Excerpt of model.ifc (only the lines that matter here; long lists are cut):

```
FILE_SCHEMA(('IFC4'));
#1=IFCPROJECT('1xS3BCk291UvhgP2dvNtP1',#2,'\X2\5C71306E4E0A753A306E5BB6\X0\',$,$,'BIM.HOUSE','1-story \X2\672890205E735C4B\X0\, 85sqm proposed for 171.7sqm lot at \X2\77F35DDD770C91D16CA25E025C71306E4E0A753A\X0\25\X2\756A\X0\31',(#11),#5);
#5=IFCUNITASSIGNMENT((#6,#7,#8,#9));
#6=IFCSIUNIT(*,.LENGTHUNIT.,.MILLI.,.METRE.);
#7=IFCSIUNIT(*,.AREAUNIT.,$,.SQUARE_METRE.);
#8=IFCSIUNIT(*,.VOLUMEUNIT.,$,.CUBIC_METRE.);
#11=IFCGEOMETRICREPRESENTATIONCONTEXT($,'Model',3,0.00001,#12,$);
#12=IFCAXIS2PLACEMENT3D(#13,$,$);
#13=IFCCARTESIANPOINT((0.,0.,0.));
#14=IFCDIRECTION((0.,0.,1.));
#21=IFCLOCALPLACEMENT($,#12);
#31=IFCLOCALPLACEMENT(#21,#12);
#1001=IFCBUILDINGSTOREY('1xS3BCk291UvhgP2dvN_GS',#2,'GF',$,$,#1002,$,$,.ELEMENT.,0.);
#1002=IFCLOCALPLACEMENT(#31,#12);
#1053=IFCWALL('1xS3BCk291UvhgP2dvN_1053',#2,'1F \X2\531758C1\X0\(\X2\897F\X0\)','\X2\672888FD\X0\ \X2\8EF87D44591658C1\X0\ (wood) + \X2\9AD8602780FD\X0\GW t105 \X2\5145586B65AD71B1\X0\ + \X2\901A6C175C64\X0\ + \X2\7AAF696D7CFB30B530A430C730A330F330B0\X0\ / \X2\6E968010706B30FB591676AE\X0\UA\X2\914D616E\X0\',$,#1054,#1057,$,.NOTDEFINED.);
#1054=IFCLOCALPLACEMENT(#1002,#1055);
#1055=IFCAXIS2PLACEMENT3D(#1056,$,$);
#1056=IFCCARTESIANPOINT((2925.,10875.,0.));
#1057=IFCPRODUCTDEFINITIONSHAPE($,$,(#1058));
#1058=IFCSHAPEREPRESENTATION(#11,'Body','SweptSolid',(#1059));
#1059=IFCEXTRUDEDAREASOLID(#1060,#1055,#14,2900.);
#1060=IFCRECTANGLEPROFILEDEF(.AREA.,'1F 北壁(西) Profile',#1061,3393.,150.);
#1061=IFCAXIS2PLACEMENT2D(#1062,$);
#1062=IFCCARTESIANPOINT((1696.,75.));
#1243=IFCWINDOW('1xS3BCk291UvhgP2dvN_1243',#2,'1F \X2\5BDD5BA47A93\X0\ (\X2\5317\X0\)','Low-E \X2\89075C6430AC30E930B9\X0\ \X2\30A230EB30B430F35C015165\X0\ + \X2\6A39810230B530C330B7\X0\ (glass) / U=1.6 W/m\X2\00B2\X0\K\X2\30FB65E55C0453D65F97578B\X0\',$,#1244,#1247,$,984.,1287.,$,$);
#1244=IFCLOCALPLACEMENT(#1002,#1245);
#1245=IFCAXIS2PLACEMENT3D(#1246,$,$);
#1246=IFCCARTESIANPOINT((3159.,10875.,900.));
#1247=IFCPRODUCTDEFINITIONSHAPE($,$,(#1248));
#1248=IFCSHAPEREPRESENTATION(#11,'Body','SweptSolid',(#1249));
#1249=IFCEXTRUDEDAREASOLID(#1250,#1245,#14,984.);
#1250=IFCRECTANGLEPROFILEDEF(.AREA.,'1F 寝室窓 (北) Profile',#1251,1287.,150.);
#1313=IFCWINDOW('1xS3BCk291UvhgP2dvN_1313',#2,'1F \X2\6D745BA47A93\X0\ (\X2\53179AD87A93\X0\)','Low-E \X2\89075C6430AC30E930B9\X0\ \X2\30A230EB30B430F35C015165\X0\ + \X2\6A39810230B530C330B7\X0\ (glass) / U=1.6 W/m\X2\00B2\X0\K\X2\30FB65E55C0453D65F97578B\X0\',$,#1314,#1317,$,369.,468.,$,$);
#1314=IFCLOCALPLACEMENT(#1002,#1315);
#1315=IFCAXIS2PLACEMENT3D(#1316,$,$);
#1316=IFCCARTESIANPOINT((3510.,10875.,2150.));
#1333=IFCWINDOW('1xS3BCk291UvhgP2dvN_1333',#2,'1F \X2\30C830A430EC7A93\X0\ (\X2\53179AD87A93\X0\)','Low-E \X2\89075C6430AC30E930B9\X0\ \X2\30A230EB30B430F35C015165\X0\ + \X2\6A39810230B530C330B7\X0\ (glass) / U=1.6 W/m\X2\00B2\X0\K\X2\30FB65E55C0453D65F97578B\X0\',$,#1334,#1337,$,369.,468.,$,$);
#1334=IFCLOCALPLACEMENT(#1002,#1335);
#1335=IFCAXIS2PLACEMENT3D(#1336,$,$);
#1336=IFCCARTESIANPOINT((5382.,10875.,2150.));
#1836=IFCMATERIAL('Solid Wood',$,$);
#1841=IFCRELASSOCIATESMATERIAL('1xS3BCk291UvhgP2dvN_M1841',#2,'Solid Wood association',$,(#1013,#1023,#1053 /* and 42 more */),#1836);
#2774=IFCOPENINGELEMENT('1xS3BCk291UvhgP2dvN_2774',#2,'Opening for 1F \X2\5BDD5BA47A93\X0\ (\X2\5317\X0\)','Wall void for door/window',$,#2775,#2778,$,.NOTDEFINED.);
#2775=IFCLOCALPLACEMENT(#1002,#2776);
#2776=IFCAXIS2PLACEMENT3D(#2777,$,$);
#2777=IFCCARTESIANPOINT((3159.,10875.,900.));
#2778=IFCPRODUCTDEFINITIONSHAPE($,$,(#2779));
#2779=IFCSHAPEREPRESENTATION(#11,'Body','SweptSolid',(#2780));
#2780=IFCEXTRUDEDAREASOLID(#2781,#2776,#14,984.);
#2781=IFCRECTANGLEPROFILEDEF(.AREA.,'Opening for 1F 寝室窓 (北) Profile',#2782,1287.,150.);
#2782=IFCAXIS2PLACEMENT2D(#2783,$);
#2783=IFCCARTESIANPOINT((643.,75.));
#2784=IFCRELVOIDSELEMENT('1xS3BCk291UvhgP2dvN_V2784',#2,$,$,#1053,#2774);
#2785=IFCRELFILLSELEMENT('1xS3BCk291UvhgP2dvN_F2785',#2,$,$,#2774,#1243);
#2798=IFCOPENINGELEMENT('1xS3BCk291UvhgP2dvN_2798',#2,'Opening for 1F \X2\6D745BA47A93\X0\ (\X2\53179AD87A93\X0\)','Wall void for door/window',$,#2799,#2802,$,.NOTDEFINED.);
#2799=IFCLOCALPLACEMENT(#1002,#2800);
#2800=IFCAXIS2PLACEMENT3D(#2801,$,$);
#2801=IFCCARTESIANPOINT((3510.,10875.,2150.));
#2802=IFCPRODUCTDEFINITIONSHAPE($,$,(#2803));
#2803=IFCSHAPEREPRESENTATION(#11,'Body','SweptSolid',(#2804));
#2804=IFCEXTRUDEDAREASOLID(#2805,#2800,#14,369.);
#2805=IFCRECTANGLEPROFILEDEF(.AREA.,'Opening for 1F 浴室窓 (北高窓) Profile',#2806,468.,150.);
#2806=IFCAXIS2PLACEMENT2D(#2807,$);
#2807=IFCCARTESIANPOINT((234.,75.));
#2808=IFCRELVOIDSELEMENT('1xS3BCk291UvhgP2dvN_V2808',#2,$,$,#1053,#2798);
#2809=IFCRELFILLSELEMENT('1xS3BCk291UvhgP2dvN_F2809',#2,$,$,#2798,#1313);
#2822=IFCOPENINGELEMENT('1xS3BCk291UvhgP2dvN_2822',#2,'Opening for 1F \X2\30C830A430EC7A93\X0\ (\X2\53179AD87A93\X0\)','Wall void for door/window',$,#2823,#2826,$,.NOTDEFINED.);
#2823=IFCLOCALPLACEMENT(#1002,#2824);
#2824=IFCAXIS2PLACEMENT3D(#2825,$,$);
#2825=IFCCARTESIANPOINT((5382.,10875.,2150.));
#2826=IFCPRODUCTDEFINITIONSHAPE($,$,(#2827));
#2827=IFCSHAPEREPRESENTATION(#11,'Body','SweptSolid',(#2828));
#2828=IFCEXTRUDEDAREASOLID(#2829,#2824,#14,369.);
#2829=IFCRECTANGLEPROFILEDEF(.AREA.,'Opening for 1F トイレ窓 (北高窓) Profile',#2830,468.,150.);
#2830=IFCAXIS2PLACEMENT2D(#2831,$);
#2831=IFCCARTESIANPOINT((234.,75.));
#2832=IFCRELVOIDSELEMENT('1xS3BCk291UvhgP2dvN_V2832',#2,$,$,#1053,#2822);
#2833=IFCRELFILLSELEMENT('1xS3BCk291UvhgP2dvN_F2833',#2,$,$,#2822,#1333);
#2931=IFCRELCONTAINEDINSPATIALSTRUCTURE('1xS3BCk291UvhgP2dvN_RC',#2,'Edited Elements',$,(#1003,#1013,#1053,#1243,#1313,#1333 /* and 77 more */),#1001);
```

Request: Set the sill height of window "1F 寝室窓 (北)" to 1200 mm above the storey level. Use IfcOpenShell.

```python
import numpy as np
import ifcopenshell
import ifcopenshell.api.geometry
import ifcopenshell.geom
import ifcopenshell.util.element
import ifcopenshell.util.placement
import ifcopenshell.util.shape
import ifcopenshell.util.unit

model = ifcopenshell.open("model.ifc")
unit_scale = ifcopenshell.util.unit.calculate_unit_scale(model)

window = model.by_guid("1xS3BCk291UvhgP2dvN_1243")
opening = window.FillsVoids[0].RelatingOpeningElement
storey = ifcopenshell.util.element.get_container(window, ifc_class="IfcBuildingStorey")
level = ifcopenshell.util.placement.get_local_placement(storey.ObjectPlacement)[2, 3]

# The opening's origin need not be at the sill, so measure its lowest point.
shape = ifcopenshell.geom.create_shape(ifcopenshell.geom.settings(), opening)
bottom = ifcopenshell.util.shape.get_shape_bottom_elevation(shape, shape.geometry) / unit_scale
dz = level + 1200.0 - bottom

shift = np.array([0.0, 0.0, dz])
# The window is not placed relative to its opening, so move both.
for product in (opening, window):
    matrix = ifcopenshell.util.placement.get_local_placement(product.ObjectPlacement)
    matrix[:3, 3] += shift
    ifcopenshell.api.geometry.edit_object_placement(model, product=product, matrix=matrix, is_si=False)

print(f"moved by {dz * unit_scale:+.3f} m")

model.write("model_rev.ifc")
```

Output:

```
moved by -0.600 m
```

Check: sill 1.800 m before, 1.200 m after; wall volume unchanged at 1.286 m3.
